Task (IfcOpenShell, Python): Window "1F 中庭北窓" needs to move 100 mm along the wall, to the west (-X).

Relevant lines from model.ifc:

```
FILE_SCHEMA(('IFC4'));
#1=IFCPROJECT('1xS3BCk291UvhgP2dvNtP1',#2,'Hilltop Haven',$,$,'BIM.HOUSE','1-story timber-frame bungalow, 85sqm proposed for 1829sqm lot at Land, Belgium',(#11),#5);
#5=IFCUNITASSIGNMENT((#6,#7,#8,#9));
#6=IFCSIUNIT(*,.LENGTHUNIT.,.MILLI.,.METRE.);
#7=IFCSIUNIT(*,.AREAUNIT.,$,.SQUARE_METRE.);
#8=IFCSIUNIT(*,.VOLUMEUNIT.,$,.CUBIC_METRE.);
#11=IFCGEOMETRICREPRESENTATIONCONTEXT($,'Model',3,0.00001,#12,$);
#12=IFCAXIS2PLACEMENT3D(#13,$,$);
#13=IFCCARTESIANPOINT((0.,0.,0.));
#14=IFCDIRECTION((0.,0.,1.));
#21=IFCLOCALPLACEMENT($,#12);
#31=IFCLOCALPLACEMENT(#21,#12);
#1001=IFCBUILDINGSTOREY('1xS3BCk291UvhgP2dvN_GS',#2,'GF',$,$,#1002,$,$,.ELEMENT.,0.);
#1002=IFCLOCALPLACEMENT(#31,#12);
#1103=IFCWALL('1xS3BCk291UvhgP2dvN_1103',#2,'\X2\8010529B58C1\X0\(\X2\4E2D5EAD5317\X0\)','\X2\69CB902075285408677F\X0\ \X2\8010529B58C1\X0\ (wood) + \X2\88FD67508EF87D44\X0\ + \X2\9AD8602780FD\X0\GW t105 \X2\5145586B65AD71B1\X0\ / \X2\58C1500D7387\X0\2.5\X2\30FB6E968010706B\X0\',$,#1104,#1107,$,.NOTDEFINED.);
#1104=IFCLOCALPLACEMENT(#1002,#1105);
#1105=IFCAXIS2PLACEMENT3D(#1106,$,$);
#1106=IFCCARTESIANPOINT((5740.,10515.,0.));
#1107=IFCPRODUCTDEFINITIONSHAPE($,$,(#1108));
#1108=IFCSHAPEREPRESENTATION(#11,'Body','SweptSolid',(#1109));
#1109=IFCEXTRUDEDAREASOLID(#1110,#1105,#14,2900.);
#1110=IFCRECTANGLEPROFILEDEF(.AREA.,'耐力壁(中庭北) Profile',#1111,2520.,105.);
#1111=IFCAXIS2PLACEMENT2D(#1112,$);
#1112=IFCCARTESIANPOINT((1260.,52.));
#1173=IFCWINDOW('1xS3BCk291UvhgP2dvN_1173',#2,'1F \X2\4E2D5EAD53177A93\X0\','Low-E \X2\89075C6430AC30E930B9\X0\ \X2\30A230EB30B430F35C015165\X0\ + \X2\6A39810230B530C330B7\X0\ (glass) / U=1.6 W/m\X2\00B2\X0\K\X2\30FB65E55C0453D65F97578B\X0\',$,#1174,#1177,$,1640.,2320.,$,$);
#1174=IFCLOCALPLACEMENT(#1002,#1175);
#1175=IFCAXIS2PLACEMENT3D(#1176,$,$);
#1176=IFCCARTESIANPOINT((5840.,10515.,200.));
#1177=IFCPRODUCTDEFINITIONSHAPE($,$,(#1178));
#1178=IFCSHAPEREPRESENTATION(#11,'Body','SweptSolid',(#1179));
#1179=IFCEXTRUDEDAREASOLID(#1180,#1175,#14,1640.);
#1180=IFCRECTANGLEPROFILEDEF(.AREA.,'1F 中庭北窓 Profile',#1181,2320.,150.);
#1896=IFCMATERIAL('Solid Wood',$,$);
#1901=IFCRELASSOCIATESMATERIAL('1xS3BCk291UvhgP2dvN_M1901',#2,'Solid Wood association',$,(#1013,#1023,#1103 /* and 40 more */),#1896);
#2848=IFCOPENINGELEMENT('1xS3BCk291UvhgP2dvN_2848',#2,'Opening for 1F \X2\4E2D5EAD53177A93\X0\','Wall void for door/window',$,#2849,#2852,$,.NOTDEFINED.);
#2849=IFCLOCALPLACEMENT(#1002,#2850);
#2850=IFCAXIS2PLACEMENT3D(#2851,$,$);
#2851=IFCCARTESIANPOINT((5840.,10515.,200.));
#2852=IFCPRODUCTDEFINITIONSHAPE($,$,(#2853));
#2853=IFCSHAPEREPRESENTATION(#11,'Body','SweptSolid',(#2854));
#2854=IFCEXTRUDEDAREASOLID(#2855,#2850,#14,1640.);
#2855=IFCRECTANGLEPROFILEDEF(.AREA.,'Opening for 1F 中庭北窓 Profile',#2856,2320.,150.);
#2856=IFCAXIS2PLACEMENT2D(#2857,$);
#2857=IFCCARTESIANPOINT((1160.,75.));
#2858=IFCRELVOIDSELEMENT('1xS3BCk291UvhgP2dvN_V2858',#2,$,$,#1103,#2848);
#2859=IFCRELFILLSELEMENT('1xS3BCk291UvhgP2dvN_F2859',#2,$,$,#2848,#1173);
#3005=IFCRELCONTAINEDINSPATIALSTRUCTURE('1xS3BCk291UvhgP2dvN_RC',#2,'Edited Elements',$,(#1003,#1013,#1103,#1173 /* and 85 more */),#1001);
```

```python
import ifcopenshell
import ifcopenshell.api.geometry
import ifcopenshell.util.placement
import ifcopenshell.util.unit

model = ifcopenshell.open("model.ifc")
unit_scale = ifcopenshell.util.unit.calculate_unit_scale(model)

window = model.by_guid("1xS3BCk291UvhgP2dvN_1173")
opening = window.FillsVoids[0].RelatingOpeningElement
wall = opening.VoidsElements[0].RelatingBuildingElement

wall_matrix = ifcopenshell.util.placement.get_local_placement(wall.ObjectPlacement)
shift = wall_matrix[:3, 0] * -0.1 / unit_scale
before = ifcopenshell.util.placement.get_local_placement(window.ObjectPlacement)[:3, 3].copy()

# The window is not placed relative to its opening, so move both.
for product in (opening, window):
    matrix = ifcopenshell.util.placement.get_local_placement(product.ObjectPlacement)
    matrix[:3, 3] += shift
    ifcopenshell.api.geometry.edit_object_placement(model, product=product, matrix=matrix, is_si=False)

after = ifcopenshell.util.placement.get_local_placement(window.ObjectPlacement)[:3, 3]
print("window moved by", (after - before).round(3) + 0.0)

model.write("model_rev.ifc")
```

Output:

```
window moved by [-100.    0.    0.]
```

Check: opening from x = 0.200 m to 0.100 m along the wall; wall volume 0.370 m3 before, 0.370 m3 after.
